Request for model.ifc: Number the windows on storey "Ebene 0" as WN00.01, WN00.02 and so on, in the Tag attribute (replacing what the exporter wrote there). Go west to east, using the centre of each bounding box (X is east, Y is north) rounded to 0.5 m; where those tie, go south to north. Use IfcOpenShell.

First a look at what the model holds.

```python
import ifcopenshell
import ifcopenshell.util.element
import ifcopenshell.util.placement

model = ifcopenshell.open("model.ifc")
print(model.schema)
storey = next(s for s in model.by_type("IfcBuildingStorey") if s.Name == "Ebene 0")
windows = [e for e in ifcopenshell.util.element.get_decomposition(storey) if e.is_a("IfcWindow")]
for e in sorted(windows, key=lambda e: e.id()):
    origin = ifcopenshell.util.placement.get_local_placement(e.ObjectPlacement)[:3, 3]
    print(e.id(), e.Tag, e.Name, origin.round(2) + 0.0, sep=" | ")
```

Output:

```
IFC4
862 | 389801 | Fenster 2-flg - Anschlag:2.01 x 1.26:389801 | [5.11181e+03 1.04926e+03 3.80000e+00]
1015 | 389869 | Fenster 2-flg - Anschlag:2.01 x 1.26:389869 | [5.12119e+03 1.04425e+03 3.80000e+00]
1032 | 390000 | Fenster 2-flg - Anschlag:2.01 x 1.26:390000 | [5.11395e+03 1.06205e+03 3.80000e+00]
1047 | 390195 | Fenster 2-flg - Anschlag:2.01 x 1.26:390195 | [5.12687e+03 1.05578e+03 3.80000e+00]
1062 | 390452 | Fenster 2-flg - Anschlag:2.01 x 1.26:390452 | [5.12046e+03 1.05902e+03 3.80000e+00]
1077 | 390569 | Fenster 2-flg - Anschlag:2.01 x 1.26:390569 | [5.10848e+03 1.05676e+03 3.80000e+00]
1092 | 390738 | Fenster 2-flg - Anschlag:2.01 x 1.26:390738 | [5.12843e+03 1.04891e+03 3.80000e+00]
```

```python
import ifcopenshell
import ifcopenshell.geom
import ifcopenshell.util.element
import ifcopenshell.util.shape

model = ifcopenshell.open("model.ifc")
settings = ifcopenshell.geom.settings()
settings.set("use-world-coords", True)


def centre(element):
    shape = ifcopenshell.geom.create_shape(settings, element)
    return ifcopenshell.util.shape.get_bbox_centroid(shape.geometry)


storey = next(s for s in model.by_type("IfcBuildingStorey") if s.Name == "Ebene 0")
windows = [e for e in ifcopenshell.util.element.get_decomposition(storey) if e.is_a("IfcWindow")]

# Insertion points can sit at a corner or the storey origin, so sort by the geometry (in metres).
centres = {e: centre(e) for e in windows}
windows.sort(key=lambda e: (round(centres[e][0] / 0.5), centres[e][1]))

for i, e in enumerate(windows, start=1):
    number = f"WN00.{i:02d}"
    e.Tag = number
    print(e.id(), number)

model.write("model_updated.ifc")
```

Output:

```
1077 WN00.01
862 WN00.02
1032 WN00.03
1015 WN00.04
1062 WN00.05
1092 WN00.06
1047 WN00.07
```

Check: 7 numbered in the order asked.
